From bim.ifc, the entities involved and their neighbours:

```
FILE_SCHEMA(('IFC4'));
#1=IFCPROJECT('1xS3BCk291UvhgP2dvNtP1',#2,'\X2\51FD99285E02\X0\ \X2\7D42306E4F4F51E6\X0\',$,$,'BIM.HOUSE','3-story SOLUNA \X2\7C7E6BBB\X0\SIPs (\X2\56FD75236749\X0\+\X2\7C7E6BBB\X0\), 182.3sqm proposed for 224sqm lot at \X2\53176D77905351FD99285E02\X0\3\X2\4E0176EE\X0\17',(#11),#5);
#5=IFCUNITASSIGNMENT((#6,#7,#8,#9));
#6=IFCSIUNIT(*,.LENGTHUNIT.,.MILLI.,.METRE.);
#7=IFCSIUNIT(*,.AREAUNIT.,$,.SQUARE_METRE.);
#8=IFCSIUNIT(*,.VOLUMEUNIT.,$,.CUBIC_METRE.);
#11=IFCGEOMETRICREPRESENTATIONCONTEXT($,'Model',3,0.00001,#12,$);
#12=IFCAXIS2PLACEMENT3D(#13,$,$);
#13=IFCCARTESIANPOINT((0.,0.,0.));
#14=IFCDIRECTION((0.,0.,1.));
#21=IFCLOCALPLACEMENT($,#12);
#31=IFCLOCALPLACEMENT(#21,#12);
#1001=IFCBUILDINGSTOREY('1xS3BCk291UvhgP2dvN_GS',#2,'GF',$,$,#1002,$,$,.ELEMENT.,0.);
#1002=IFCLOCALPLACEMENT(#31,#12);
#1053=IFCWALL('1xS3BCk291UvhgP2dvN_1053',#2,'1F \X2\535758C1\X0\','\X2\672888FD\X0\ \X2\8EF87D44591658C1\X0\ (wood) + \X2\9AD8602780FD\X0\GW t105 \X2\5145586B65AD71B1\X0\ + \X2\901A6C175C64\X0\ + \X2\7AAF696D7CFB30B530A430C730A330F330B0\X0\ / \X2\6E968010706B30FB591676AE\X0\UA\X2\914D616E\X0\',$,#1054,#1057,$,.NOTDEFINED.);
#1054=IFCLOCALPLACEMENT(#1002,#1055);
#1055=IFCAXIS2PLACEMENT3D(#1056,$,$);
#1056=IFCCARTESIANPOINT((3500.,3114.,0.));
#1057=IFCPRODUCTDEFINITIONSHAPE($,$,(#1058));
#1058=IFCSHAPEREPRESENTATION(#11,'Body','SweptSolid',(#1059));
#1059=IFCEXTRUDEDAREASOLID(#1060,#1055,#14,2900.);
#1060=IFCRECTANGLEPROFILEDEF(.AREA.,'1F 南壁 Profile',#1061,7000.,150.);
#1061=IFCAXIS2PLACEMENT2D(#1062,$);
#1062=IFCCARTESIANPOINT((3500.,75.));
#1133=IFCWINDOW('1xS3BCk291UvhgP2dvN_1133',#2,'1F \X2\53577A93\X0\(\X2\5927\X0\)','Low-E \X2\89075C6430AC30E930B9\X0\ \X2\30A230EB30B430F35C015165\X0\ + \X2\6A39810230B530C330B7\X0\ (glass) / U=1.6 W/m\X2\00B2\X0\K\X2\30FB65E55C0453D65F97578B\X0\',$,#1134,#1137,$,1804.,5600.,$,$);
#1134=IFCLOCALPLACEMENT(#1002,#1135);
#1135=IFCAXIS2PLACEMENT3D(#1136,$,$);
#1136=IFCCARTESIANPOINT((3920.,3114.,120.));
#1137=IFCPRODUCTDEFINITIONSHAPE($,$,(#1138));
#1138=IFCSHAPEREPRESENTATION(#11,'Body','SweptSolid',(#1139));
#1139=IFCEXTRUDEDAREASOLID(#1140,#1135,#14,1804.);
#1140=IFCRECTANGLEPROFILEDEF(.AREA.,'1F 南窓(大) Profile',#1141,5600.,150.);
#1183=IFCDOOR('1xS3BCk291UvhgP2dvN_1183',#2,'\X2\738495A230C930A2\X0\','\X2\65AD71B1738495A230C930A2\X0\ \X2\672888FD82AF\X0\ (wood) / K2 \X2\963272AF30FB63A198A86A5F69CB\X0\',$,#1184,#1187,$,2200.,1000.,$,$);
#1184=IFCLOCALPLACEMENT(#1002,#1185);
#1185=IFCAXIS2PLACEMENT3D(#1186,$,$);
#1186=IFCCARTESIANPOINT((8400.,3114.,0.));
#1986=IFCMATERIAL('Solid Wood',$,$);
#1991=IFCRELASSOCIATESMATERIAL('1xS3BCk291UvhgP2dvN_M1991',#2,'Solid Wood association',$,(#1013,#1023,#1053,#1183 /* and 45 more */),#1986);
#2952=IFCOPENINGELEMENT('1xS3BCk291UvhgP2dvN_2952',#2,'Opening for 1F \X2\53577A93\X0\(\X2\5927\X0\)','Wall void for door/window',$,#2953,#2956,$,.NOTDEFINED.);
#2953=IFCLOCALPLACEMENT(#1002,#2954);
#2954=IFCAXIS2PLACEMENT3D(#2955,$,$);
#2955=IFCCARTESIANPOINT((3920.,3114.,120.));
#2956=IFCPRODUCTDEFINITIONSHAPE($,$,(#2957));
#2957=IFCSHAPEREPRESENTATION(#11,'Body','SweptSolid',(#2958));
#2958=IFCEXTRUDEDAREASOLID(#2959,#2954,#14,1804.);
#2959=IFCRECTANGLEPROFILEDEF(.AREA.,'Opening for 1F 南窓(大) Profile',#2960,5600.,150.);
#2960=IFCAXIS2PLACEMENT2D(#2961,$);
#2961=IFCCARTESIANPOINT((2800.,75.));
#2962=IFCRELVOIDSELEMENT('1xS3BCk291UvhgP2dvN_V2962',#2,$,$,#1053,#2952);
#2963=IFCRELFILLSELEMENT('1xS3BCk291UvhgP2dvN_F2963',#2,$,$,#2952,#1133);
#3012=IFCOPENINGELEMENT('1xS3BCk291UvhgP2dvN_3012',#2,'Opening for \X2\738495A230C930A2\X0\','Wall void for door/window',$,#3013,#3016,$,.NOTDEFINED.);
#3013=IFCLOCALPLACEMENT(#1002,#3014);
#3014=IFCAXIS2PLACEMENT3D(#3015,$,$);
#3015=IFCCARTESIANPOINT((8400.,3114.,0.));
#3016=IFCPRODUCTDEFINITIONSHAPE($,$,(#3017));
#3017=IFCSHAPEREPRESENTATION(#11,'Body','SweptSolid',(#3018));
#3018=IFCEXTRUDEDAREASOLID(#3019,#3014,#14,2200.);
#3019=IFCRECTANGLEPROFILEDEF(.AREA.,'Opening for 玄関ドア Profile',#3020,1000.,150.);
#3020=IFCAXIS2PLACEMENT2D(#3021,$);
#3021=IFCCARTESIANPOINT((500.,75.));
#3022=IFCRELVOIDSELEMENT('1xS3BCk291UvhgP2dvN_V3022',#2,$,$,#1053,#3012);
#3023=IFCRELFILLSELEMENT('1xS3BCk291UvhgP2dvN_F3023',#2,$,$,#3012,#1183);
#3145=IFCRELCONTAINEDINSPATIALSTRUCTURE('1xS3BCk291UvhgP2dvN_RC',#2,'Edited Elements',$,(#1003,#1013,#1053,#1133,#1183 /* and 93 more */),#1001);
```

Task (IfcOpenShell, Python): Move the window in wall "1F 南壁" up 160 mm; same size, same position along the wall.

```python
import numpy as np
import ifcopenshell
import ifcopenshell.api.geometry
import ifcopenshell.util.placement
import ifcopenshell.util.unit

model = ifcopenshell.open("bim.ifc")
unit_scale = ifcopenshell.util.unit.calculate_unit_scale(model)

window = model.by_guid("1xS3BCk291UvhgP2dvN_1133")
opening = window.FillsVoids[0].RelatingOpeningElement
dz = 160.0

shift = np.array([0.0, 0.0, dz])
# The window is not placed relative to its opening, so move both.
for product in (opening, window):
    matrix = ifcopenshell.util.placement.get_local_placement(product.ObjectPlacement)
    matrix[:3, 3] += shift
    ifcopenshell.api.geometry.edit_object_placement(model, product=product, matrix=matrix, is_si=False)

print(f"moved by {dz * unit_scale:+.3f} m")

model.write("bim-out.ifc")
```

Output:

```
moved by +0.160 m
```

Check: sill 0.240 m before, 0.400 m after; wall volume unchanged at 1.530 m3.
